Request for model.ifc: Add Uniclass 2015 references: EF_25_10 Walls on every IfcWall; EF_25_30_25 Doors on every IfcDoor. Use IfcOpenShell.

First a look at what the model holds.

```python
import ifcopenshell

model = ifcopenshell.open("model.ifc")
print(model.schema)
print("classifications:", [c.Name for c in model.by_type("IfcClassification")])
for ifc_class in ("IfcDoor", "IfcRoof", "IfcStair", "IfcWall", "IfcWindow"):
    print(ifc_class, len(model.by_type(ifc_class)))
```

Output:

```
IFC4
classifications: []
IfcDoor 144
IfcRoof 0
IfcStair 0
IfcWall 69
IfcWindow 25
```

```python
import ifcopenshell
import ifcopenshell.api.classification

model = ifcopenshell.open("model.ifc")

system = ifcopenshell.api.classification.add_classification(model, classification="Uniclass 2015")

codes = {
    "IfcWall": ("EF_25_10", "Walls"),
    "IfcDoor": ("EF_25_30_25", "Doors"),
}
for ifc_class, (code, name) in codes.items():
    products = model.by_type(ifc_class)
    ifcopenshell.api.classification.add_reference(
        model, products=products, classification=system, identification=code, name=name
    )
    print(code, len(products))

model.write("model_updated.ifc")
```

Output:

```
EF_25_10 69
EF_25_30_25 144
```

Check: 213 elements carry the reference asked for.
